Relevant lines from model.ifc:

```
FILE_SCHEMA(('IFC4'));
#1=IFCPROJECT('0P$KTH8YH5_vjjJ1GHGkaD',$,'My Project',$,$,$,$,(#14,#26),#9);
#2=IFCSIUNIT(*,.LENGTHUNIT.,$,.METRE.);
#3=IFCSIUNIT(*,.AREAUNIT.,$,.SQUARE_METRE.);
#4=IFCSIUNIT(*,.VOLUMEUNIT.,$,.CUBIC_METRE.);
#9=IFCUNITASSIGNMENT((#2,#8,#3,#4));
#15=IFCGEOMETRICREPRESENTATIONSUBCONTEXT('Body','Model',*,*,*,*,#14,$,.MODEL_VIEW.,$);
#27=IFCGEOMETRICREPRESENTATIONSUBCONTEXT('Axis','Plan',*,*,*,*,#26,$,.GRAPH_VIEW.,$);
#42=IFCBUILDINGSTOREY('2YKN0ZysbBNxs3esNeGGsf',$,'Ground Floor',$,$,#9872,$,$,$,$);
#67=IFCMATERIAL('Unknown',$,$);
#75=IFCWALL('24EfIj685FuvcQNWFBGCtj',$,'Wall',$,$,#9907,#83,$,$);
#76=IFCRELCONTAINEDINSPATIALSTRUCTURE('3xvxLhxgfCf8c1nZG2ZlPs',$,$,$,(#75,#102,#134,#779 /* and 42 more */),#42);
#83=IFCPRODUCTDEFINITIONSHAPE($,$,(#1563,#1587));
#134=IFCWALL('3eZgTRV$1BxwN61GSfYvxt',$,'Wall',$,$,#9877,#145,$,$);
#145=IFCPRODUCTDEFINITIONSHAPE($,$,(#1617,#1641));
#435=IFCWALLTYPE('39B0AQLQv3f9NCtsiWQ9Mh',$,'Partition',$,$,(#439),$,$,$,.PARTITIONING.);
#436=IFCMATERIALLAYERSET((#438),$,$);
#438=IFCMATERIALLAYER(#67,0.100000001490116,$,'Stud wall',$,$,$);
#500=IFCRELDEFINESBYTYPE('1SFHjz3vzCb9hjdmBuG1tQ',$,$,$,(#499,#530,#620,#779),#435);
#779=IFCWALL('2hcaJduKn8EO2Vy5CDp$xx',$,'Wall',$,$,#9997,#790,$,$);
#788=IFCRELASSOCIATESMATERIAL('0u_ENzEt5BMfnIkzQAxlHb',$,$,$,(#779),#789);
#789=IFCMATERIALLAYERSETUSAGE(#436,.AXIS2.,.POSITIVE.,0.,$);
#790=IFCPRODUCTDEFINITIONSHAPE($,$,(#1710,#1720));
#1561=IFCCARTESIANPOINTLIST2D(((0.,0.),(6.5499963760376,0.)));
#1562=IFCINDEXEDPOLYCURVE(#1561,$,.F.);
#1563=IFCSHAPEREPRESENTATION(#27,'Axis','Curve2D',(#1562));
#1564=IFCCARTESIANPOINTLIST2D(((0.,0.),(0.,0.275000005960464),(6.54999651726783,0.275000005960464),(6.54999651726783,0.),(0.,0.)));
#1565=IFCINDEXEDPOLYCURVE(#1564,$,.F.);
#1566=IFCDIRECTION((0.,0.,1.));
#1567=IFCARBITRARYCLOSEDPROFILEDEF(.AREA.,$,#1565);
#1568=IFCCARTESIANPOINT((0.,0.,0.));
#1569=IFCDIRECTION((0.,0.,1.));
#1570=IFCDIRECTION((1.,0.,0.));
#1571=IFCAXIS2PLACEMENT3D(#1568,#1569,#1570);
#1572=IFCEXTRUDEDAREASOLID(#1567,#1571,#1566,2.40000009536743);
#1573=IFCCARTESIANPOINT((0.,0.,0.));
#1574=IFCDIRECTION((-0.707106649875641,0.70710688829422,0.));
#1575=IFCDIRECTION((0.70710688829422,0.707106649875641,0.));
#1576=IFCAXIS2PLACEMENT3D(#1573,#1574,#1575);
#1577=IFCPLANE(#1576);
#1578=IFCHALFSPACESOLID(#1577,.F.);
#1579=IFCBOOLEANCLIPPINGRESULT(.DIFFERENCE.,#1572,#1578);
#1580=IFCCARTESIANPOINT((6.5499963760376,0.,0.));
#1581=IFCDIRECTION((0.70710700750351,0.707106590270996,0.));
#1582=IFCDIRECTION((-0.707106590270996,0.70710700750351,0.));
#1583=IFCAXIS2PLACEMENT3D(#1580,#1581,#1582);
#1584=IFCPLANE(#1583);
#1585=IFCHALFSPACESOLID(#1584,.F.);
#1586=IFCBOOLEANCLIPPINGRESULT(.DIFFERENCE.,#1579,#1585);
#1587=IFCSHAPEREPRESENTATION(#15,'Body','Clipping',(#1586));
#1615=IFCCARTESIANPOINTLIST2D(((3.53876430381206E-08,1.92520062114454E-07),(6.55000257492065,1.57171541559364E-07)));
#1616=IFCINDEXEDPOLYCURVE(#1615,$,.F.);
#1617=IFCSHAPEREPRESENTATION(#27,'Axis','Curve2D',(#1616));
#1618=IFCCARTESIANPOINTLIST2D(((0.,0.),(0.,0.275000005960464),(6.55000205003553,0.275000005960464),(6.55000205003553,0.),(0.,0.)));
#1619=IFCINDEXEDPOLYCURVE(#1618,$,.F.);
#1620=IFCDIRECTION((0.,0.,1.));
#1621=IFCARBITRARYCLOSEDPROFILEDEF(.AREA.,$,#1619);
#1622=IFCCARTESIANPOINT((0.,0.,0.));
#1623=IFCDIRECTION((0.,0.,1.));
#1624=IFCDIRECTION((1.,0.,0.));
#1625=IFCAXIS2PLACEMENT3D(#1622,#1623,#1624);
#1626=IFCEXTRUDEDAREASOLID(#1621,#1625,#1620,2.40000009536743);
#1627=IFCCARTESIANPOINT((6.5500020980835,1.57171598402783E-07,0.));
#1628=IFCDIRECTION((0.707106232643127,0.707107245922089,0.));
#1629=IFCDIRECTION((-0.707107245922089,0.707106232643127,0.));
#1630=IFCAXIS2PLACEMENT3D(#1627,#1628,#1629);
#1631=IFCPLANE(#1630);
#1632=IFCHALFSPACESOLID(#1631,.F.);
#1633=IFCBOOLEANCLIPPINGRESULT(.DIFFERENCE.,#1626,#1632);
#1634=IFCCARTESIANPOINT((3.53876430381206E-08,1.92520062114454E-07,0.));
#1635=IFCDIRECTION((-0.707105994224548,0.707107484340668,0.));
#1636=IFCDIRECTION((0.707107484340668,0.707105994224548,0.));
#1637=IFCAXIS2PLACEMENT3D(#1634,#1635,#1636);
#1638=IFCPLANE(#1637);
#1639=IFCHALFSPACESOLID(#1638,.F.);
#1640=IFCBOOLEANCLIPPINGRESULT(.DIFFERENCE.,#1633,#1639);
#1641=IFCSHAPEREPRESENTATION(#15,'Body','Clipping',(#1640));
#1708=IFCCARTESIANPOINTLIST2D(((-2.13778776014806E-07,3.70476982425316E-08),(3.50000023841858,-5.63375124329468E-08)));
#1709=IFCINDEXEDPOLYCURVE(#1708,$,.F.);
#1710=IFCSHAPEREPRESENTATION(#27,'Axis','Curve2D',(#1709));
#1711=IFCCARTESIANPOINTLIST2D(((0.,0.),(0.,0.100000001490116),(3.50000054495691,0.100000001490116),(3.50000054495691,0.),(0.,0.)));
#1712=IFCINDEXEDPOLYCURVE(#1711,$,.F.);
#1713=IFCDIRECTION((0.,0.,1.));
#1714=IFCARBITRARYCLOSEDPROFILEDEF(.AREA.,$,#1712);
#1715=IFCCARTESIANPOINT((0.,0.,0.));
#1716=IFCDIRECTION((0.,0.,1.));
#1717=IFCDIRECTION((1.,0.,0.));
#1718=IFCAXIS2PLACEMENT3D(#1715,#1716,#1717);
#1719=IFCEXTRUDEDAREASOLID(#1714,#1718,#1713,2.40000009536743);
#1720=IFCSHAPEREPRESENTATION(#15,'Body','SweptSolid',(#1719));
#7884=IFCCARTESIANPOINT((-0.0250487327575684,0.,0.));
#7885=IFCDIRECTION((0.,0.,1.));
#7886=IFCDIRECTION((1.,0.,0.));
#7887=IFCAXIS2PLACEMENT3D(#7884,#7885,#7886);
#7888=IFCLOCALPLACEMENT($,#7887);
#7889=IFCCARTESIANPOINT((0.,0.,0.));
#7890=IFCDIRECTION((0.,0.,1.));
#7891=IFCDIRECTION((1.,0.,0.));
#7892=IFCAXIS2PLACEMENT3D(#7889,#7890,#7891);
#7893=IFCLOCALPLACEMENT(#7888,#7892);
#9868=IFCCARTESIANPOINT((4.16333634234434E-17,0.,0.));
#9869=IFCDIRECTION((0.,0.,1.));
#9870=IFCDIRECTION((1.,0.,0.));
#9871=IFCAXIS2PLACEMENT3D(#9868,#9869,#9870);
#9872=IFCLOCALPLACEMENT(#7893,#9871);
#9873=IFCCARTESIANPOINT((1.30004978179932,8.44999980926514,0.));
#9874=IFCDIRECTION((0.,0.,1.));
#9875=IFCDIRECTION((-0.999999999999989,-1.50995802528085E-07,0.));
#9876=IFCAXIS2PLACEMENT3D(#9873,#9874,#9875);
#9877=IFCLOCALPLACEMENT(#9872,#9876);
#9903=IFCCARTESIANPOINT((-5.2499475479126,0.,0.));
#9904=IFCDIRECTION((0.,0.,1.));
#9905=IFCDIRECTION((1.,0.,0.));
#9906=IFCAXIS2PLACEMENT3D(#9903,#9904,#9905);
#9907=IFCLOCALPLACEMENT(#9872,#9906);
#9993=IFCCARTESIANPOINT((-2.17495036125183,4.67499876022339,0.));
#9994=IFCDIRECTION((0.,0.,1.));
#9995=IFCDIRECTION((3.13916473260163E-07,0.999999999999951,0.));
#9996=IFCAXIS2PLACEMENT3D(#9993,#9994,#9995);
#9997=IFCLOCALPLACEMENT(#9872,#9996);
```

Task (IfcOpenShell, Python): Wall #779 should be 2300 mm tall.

```python
import ifcopenshell
import ifcopenshell.geom
import ifcopenshell.util.representation
import ifcopenshell.util.shape
import ifcopenshell.util.unit

model = ifcopenshell.open("model.ifc")
unit_scale = ifcopenshell.util.unit.calculate_unit_scale(model)
settings = ifcopenshell.geom.settings()


def volume(element):
    """Net volume in cubic metres, openings subtracted."""
    shape = ifcopenshell.geom.create_shape(settings, element)
    return ifcopenshell.util.shape.get_volume(shape.geometry)


wall = model.by_guid("2hcaJduKn8EO2Vy5CDp$xx")
before = volume(wall)

body = ifcopenshell.util.representation.get_representation(wall, "Model", "Body")
solid = body.Items[0]
old_height = solid.Depth
solid.Depth = 2.3 / unit_scale
after = volume(wall)

print(f"height {old_height:g} -> {solid.Depth:g}, volume {before:.3f} -> {after:.3f} m3")

model.write("model_edited.ifc")
```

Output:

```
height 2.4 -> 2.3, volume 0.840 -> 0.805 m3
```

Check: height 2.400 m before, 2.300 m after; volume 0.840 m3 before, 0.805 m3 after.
